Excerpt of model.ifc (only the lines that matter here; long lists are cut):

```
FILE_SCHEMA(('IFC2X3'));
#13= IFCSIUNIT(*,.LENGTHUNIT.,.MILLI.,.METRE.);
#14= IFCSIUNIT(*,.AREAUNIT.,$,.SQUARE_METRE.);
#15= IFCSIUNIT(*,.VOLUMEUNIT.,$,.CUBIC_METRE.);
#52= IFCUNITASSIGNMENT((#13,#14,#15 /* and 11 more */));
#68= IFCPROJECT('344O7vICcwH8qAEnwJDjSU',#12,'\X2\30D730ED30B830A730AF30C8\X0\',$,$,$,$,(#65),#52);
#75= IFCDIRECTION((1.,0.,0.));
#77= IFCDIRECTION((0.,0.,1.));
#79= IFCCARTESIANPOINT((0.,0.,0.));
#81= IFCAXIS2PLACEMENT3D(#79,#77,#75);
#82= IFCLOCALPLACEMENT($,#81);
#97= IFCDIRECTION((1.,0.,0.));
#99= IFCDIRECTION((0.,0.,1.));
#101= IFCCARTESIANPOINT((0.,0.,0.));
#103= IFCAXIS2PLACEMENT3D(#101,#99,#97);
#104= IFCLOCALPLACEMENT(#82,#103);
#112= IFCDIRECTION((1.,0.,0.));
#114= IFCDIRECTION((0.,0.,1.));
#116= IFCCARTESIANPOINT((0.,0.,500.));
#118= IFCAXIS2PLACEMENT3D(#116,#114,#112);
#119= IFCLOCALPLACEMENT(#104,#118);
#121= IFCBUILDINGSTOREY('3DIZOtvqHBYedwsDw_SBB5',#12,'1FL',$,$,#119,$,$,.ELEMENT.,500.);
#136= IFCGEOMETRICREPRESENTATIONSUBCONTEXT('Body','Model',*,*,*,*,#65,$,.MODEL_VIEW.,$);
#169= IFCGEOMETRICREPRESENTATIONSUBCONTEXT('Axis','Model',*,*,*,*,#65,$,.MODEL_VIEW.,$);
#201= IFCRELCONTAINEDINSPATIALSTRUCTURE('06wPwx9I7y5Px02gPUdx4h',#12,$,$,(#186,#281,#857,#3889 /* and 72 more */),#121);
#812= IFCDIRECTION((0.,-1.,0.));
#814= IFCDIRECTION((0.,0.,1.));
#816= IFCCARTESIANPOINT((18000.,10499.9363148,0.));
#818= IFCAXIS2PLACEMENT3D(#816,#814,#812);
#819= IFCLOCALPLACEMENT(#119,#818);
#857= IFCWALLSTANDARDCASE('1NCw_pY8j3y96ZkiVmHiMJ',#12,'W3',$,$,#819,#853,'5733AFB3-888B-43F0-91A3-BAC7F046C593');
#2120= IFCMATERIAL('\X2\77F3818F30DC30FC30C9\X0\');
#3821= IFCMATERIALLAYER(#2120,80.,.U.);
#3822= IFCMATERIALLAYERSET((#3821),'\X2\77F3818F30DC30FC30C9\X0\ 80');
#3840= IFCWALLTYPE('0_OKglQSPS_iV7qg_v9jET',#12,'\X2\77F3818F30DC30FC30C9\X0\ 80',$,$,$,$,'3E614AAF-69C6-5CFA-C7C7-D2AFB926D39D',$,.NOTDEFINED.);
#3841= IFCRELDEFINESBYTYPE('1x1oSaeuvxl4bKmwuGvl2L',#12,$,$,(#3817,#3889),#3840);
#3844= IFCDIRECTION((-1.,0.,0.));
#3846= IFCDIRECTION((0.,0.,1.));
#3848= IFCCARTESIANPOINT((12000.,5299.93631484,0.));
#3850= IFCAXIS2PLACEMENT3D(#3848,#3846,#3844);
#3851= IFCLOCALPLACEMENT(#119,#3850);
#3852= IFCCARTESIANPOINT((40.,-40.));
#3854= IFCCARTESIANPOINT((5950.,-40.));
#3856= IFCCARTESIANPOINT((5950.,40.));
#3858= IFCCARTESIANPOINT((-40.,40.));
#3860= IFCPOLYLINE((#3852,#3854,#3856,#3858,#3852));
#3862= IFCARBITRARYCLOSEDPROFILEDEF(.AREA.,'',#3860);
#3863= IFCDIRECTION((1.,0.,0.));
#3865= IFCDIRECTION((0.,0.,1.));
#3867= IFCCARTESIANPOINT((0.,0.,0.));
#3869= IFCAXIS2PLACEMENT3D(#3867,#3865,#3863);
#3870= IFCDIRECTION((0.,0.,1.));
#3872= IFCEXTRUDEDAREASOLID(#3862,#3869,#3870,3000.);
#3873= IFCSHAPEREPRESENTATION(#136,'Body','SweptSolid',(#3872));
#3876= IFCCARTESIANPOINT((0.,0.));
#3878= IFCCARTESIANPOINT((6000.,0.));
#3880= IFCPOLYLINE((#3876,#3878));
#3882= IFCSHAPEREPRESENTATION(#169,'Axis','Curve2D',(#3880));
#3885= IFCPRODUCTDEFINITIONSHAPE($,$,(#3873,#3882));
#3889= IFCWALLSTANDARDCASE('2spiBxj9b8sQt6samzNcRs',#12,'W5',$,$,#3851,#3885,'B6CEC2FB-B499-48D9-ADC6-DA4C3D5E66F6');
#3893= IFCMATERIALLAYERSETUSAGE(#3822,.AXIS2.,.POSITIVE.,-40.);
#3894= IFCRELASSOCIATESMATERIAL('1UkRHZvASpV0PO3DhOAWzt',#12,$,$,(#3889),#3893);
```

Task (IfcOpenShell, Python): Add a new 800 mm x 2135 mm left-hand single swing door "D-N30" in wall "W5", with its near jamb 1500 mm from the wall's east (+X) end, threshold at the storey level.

```python
import numpy as np
import ifcopenshell
import ifcopenshell.api.feature
import ifcopenshell.api.geometry
import ifcopenshell.api.root
import ifcopenshell.api.spatial
import ifcopenshell.api.type
import ifcopenshell.geom
import ifcopenshell.util.element
import ifcopenshell.util.placement
import ifcopenshell.util.representation
import ifcopenshell.util.shape
import ifcopenshell.util.unit

model = ifcopenshell.open("model.ifc")
unit_scale = ifcopenshell.util.unit.calculate_unit_scale(model)
settings = ifcopenshell.geom.settings()


def volume(element):
    """Net volume in cubic metres, openings subtracted."""
    shape = ifcopenshell.geom.create_shape(settings, element)
    return ifcopenshell.util.shape.get_volume(shape.geometry)


wall = model.by_guid("2spiBxj9b8sQt6samzNcRs")
storey = ifcopenshell.util.element.get_container(wall, ifc_class="IfcBuildingStorey")
context = ifcopenshell.util.representation.get_context(model, "Model", "Body", "MODEL_VIEW")
before = volume(wall)

width, height, from_end, sill = 0.8, 2.135, 1.5, 0.0  # metres

# The wall runs along its own X axis, and the end named is its -X end.
wall_shape = ifcopenshell.geom.create_shape(settings, wall)
x, y, z = ifcopenshell.util.shape.get_vertices(wall_shape.geometry).T
start = x.min() + from_end
face, thickness = float(y.min()), float(y.max() - y.min())
wall_matrix = ifcopenshell.util.placement.get_local_placement(wall.ObjectPlacement)
level = ifcopenshell.util.placement.get_local_placement(storey.ObjectPlacement)[2, 3]


def in_wall(x, y):
    """Placement at x, y metres in the wall's axes, at sill height."""
    matrix = wall_matrix.copy()
    matrix[:, 3] = wall_matrix @ np.array([x / unit_scale, y / unit_scale, 0.0, 1.0])
    matrix[2, 3] = level + sill / unit_scale
    return matrix


# Opening: a box that overshoots both wall faces by 50 mm.
opening = ifcopenshell.api.root.create_entity(model, ifc_class="IfcOpeningElement")
box = ifcopenshell.api.geometry.add_wall_representation(
    model, context=context, length=width, height=height, thickness=thickness + 0.1
)
ifcopenshell.api.geometry.assign_representation(model, product=opening, representation=box)
ifcopenshell.api.geometry.edit_object_placement(model, product=opening, matrix=in_wall(start, face - 0.05), is_si=False)
ifcopenshell.api.feature.add_feature(model, feature=opening, element=wall)

door = ifcopenshell.api.root.create_entity(model, ifc_class="IfcDoor", name="D-N30")
door.OverallWidth, door.OverallHeight = width / unit_scale, height / unit_scale
body = ifcopenshell.api.geometry.add_door_representation(
    model,
    context=context,
    overall_width=door.OverallWidth,
    overall_height=door.OverallHeight,
    operation_type="SINGLE_SWING_LEFT",
    lining_properties={"LiningDepth": thickness / unit_scale, "ThresholdDepth": thickness / unit_scale},
)
ifcopenshell.api.geometry.assign_representation(model, product=door, representation=body)
ifcopenshell.api.spatial.assign_container(model, products=[door], relating_structure=storey)
fills = ifcopenshell.api.feature.add_filling(model, opening=opening, element=door)
fills.OwnerHistory = door.OwnerHistory  # required in IFC2X3

# IFC2X3 keeps the operation on the door style.
style = ifcopenshell.api.root.create_entity(model, ifc_class="IfcDoorStyle", name="D-N30")
style.OperationType, style.ConstructionType = "SINGLE_SWING_LEFT", "NOTDEFINED"
style.ParameterTakesPrecedence = style.Sizeable = False
ifcopenshell.api.type.assign_type(model, related_objects=[door], relating_type=style)

# The lining spans the wall, so the door starts at the wall face.
ifcopenshell.api.geometry.edit_object_placement(model, product=door, matrix=in_wall(start, face), is_si=False)

after = volume(wall)

print(f"wall volume {before:.3f} -> {after:.3f} m3")

model.write("model_v2.ifc")
```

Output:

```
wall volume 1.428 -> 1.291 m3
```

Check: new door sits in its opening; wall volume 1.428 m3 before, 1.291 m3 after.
